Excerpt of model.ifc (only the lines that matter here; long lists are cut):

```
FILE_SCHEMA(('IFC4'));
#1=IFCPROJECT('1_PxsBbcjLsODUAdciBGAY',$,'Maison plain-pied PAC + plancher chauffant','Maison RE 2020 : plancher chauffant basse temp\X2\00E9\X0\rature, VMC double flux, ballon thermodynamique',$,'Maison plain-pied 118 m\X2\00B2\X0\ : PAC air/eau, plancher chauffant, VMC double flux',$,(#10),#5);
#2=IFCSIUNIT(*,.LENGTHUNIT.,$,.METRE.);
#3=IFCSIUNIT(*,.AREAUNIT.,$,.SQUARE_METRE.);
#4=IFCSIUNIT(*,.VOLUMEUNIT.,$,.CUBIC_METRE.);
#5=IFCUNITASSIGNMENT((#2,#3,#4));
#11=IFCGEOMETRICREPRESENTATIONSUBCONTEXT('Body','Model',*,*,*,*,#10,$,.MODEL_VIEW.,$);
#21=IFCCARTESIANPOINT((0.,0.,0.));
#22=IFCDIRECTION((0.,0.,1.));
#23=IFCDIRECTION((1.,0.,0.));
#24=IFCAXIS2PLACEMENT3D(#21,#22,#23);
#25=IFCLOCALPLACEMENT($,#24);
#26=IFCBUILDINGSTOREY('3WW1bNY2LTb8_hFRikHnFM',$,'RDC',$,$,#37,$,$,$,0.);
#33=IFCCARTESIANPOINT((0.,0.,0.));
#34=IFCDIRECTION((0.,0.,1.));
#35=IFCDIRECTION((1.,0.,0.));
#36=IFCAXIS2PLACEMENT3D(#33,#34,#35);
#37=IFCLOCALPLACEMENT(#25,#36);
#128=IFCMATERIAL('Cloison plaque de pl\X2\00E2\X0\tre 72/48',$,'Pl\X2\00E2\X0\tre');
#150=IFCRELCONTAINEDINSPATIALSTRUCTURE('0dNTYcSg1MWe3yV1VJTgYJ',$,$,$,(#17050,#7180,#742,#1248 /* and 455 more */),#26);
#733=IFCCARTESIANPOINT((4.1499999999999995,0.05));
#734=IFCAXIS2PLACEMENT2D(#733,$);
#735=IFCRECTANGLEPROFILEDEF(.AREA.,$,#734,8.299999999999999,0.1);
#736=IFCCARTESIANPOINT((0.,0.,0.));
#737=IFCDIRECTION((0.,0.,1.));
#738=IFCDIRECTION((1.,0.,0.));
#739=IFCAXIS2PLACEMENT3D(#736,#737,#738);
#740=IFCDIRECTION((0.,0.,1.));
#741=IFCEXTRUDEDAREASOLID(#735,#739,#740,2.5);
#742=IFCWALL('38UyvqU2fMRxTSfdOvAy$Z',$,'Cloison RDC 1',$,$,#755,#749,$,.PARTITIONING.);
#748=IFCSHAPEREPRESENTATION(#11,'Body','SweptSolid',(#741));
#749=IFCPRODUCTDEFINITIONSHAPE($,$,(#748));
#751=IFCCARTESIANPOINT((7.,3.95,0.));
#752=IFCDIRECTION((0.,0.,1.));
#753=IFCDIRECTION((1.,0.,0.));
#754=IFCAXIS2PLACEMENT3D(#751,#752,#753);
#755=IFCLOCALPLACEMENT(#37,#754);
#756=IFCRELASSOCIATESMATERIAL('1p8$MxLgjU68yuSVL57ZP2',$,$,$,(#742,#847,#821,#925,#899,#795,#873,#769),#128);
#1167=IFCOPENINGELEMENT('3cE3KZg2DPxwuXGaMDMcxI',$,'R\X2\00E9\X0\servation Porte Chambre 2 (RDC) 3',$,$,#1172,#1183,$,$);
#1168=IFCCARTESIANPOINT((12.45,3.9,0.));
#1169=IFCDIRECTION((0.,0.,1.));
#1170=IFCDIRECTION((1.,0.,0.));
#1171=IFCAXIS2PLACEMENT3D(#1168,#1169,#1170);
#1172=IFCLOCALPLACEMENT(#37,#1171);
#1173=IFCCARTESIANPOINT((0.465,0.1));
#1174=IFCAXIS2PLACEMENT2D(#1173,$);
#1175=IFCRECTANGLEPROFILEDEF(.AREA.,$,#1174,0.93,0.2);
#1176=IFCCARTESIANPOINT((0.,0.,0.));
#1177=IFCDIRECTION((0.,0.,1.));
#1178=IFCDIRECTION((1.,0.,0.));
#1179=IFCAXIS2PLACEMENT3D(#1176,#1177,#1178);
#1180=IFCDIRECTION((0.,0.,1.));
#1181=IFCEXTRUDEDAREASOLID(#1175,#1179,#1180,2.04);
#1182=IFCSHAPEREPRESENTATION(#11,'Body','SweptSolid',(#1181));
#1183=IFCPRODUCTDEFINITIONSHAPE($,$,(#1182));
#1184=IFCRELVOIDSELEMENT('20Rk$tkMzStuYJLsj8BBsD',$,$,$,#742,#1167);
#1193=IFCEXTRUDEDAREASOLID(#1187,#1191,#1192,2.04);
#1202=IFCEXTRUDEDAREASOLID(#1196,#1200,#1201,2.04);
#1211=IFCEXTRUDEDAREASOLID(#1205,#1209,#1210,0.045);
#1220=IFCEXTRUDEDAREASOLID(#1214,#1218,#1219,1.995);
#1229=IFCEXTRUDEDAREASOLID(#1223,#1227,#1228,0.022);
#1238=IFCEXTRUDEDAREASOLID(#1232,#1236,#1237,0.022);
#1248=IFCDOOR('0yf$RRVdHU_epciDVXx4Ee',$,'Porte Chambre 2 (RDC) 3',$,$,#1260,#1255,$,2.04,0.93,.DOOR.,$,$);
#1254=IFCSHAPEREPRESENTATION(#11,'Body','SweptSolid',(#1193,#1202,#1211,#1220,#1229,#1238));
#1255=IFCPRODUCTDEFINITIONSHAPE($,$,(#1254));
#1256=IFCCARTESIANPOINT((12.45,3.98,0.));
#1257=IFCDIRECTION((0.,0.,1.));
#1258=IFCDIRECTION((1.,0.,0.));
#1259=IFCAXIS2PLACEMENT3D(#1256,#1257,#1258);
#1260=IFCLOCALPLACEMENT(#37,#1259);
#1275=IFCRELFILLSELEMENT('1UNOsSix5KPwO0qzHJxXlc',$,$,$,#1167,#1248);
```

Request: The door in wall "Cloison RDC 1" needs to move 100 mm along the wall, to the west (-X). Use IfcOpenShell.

```python
import ifcopenshell
import ifcopenshell.api.geometry
import ifcopenshell.util.placement
import ifcopenshell.util.unit

model = ifcopenshell.open("model.ifc")
unit_scale = ifcopenshell.util.unit.calculate_unit_scale(model)

door = model.by_id(1248)
opening = door.FillsVoids[0].RelatingOpeningElement
wall = opening.VoidsElements[0].RelatingBuildingElement

wall_matrix = ifcopenshell.util.placement.get_local_placement(wall.ObjectPlacement)
shift = wall_matrix[:3, 0] * -0.1 / unit_scale
before = ifcopenshell.util.placement.get_local_placement(door.ObjectPlacement)[:3, 3].copy()

# The door is not placed relative to its opening, so move both.
for product in (opening, door):
    matrix = ifcopenshell.util.placement.get_local_placement(product.ObjectPlacement)
    matrix[:3, 3] += shift
    ifcopenshell.api.geometry.edit_object_placement(model, product=product, matrix=matrix, is_si=False)

after = ifcopenshell.util.placement.get_local_placement(door.ObjectPlacement)[:3, 3]
print("door moved by", (after - before).round(3) + 0.0)

model.write("model_edited.ifc")
```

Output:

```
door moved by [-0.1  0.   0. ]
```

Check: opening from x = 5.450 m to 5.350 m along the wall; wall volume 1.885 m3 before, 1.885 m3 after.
